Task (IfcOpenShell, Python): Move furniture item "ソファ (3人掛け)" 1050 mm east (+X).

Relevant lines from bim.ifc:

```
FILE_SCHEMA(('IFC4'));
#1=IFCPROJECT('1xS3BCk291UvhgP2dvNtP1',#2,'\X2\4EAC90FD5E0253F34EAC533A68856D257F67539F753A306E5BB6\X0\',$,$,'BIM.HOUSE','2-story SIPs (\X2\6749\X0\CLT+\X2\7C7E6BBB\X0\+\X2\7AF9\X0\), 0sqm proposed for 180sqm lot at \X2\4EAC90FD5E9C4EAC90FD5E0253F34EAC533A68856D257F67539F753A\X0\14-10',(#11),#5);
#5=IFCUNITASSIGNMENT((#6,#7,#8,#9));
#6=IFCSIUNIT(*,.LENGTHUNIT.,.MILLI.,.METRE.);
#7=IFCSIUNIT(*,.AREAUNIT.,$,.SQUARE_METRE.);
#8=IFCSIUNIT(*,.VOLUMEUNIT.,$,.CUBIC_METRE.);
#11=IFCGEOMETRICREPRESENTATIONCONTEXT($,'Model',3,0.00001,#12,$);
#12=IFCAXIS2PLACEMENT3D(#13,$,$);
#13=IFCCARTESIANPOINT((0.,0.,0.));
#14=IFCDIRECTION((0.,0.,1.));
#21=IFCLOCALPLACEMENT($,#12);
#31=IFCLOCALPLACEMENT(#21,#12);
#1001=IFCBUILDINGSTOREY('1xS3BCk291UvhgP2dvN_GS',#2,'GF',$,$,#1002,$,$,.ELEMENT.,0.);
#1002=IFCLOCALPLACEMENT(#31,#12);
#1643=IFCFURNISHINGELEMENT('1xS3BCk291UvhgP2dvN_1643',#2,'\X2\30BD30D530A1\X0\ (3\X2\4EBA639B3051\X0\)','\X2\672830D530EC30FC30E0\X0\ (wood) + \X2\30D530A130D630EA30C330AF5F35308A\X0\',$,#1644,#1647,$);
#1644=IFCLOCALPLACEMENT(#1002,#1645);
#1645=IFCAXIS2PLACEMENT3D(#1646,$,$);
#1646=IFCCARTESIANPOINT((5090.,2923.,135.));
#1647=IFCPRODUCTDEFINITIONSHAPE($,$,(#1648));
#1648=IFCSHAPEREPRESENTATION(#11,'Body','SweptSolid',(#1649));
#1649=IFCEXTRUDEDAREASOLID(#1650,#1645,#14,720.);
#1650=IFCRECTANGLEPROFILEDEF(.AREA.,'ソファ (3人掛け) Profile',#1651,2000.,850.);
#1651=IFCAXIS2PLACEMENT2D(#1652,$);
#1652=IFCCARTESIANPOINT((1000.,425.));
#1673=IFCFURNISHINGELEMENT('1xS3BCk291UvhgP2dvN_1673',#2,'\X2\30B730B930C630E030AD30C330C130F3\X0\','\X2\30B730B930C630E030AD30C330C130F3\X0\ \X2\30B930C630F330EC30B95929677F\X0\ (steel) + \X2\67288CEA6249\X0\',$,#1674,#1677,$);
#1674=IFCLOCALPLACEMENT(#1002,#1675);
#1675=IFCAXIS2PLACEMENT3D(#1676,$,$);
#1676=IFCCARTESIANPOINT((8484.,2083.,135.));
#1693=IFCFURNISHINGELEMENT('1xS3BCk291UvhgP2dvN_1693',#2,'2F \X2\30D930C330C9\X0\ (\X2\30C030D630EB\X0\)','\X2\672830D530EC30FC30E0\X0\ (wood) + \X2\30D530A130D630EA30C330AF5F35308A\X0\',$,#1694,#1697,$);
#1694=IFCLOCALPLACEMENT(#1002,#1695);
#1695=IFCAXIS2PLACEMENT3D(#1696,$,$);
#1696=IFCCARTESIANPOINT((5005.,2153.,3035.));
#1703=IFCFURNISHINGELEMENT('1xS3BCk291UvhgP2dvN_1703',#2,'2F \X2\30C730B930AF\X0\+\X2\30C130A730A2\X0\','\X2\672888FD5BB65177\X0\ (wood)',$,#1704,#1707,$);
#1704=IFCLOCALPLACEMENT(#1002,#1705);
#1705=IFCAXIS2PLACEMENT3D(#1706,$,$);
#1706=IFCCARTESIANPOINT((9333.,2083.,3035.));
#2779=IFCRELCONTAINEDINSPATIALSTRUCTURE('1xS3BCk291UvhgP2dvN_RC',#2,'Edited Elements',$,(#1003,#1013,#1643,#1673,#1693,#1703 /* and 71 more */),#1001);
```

```python
import ifcopenshell
import ifcopenshell.api.geometry
import ifcopenshell.util.placement
import ifcopenshell.util.unit

model = ifcopenshell.open("bim.ifc")
unit_scale = ifcopenshell.util.unit.calculate_unit_scale(model)

item = model.by_guid("1xS3BCk291UvhgP2dvN_1643")
matrix = ifcopenshell.util.placement.get_local_placement(item.ObjectPlacement)
matrix[0, 3] += 1.05 / unit_scale
ifcopenshell.api.geometry.edit_object_placement(model, product=item, matrix=matrix, is_si=False)

print(ifcopenshell.util.placement.get_local_placement(item.ObjectPlacement).round(3) + 0.0)

model.write("bim-out.ifc")
```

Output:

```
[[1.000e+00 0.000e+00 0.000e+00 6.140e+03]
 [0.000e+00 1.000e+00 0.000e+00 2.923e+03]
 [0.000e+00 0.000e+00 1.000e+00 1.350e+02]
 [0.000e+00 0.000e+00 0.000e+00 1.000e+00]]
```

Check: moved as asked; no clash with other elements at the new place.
